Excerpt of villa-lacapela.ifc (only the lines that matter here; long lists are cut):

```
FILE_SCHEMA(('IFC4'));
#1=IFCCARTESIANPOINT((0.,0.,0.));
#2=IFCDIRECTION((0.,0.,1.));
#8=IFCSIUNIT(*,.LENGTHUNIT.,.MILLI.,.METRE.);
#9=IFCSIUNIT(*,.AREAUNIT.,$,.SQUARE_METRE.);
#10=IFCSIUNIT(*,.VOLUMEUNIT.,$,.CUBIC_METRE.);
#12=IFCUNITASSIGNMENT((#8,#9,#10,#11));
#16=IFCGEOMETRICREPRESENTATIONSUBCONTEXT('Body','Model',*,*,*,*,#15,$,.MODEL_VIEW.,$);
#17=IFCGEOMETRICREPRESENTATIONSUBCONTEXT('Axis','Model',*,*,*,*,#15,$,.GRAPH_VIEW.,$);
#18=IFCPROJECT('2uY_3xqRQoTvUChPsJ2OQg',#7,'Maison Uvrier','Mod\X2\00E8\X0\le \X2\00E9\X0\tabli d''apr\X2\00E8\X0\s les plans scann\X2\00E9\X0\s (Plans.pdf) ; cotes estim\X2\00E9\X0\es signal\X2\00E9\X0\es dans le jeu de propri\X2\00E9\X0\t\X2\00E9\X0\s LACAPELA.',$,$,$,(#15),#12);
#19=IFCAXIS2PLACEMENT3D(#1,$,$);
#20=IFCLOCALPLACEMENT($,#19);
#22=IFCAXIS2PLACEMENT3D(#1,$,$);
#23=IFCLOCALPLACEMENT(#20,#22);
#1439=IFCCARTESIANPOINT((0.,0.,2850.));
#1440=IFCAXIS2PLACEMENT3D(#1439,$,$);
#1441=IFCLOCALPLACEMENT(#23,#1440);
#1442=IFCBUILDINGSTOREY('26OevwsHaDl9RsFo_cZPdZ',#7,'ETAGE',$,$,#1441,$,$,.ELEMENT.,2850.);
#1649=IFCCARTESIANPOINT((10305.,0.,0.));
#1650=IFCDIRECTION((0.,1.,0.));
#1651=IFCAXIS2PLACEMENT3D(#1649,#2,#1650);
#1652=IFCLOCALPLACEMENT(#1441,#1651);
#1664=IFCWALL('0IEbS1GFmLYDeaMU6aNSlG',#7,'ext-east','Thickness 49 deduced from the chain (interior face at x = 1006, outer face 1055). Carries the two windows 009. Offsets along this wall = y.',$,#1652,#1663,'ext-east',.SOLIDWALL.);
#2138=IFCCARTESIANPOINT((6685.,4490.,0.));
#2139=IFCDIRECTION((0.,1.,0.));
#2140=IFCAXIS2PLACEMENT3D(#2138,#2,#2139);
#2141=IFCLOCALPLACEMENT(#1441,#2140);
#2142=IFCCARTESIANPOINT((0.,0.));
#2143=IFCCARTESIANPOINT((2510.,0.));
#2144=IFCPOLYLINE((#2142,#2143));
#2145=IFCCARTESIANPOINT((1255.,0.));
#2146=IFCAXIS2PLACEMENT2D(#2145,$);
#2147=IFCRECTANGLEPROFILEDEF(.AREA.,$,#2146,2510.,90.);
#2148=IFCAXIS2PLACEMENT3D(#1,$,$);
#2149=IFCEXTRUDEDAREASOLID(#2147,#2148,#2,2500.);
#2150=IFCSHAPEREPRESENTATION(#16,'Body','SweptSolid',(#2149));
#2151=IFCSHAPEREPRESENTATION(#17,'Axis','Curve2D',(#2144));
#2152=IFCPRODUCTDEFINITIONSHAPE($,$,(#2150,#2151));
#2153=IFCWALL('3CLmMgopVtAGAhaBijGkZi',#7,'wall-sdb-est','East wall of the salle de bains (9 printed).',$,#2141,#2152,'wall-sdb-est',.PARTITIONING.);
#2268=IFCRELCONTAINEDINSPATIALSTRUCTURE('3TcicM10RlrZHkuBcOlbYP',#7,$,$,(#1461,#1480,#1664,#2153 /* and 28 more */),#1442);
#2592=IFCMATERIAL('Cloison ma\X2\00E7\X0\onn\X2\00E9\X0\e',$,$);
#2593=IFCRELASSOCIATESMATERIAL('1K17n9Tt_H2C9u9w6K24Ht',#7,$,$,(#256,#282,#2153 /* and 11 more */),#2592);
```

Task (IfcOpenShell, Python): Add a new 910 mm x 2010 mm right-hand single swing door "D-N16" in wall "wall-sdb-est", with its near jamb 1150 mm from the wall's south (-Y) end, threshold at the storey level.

```python
import numpy as np
import ifcopenshell
import ifcopenshell.api.feature
import ifcopenshell.api.geometry
import ifcopenshell.api.root
import ifcopenshell.api.spatial
import ifcopenshell.geom
import ifcopenshell.util.element
import ifcopenshell.util.placement
import ifcopenshell.util.representation
import ifcopenshell.util.shape
import ifcopenshell.util.unit

model = ifcopenshell.open("villa-lacapela.ifc")
unit_scale = ifcopenshell.util.unit.calculate_unit_scale(model)
settings = ifcopenshell.geom.settings()


def volume(element):
    """Net volume in cubic metres, openings subtracted."""
    shape = ifcopenshell.geom.create_shape(settings, element)
    return ifcopenshell.util.shape.get_volume(shape.geometry)


wall = model.by_guid("3CLmMgopVtAGAhaBijGkZi")
storey = ifcopenshell.util.element.get_container(wall, ifc_class="IfcBuildingStorey")
context = ifcopenshell.util.representation.get_context(model, "Model", "Body", "MODEL_VIEW")
before = volume(wall)

width, height, from_end, sill = 0.91, 2.01, 1.15, 0.0  # metres

# The wall runs along its own X axis, and the end named is its -X end.
wall_shape = ifcopenshell.geom.create_shape(settings, wall)
x, y, z = ifcopenshell.util.shape.get_vertices(wall_shape.geometry).T
start = x.min() + from_end
face, thickness = float(y.min()), float(y.max() - y.min())
wall_matrix = ifcopenshell.util.placement.get_local_placement(wall.ObjectPlacement)
level = ifcopenshell.util.placement.get_local_placement(storey.ObjectPlacement)[2, 3]


def in_wall(x, y):
    """Placement at x, y metres in the wall's axes, at sill height."""
    matrix = wall_matrix.copy()
    matrix[:, 3] = wall_matrix @ np.array([x / unit_scale, y / unit_scale, 0.0, 1.0])
    matrix[2, 3] = level + sill / unit_scale
    return matrix


# Opening: a box that overshoots both wall faces by 50 mm.
opening = ifcopenshell.api.root.create_entity(model, ifc_class="IfcOpeningElement", predefined_type="OPENING")
box = ifcopenshell.api.geometry.add_wall_representation(
    model, context=context, length=width, height=height, thickness=thickness + 0.1
)
ifcopenshell.api.geometry.assign_representation(model, product=opening, representation=box)
ifcopenshell.api.geometry.edit_object_placement(model, product=opening, matrix=in_wall(start, face - 0.05), is_si=False)
ifcopenshell.api.feature.add_feature(model, feature=opening, element=wall)

door = ifcopenshell.api.root.create_entity(model, ifc_class="IfcDoor", name="D-N16", predefined_type="DOOR")
door.OverallWidth, door.OverallHeight = width / unit_scale, height / unit_scale
door.OperationType = "SINGLE_SWING_RIGHT"
body = ifcopenshell.api.geometry.add_door_representation(
    model,
    context=context,
    overall_width=door.OverallWidth,
    overall_height=door.OverallHeight,
    operation_type="SINGLE_SWING_RIGHT",
    lining_properties={"LiningDepth": thickness / unit_scale, "ThresholdDepth": thickness / unit_scale},
)
ifcopenshell.api.geometry.assign_representation(model, product=door, representation=body)
ifcopenshell.api.spatial.assign_container(model, products=[door], relating_structure=storey)
ifcopenshell.api.feature.add_filling(model, opening=opening, element=door)

# The lining spans the wall, so the door starts at the wall face.
ifcopenshell.api.geometry.edit_object_placement(model, product=door, matrix=in_wall(start, face), is_si=False)

after = volume(wall)

print(f"wall volume {before:.3f} -> {after:.3f} m3")

model.write("villa-lacapela_v2.ifc")
```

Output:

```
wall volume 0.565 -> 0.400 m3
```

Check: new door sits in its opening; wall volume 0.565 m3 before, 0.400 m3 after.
